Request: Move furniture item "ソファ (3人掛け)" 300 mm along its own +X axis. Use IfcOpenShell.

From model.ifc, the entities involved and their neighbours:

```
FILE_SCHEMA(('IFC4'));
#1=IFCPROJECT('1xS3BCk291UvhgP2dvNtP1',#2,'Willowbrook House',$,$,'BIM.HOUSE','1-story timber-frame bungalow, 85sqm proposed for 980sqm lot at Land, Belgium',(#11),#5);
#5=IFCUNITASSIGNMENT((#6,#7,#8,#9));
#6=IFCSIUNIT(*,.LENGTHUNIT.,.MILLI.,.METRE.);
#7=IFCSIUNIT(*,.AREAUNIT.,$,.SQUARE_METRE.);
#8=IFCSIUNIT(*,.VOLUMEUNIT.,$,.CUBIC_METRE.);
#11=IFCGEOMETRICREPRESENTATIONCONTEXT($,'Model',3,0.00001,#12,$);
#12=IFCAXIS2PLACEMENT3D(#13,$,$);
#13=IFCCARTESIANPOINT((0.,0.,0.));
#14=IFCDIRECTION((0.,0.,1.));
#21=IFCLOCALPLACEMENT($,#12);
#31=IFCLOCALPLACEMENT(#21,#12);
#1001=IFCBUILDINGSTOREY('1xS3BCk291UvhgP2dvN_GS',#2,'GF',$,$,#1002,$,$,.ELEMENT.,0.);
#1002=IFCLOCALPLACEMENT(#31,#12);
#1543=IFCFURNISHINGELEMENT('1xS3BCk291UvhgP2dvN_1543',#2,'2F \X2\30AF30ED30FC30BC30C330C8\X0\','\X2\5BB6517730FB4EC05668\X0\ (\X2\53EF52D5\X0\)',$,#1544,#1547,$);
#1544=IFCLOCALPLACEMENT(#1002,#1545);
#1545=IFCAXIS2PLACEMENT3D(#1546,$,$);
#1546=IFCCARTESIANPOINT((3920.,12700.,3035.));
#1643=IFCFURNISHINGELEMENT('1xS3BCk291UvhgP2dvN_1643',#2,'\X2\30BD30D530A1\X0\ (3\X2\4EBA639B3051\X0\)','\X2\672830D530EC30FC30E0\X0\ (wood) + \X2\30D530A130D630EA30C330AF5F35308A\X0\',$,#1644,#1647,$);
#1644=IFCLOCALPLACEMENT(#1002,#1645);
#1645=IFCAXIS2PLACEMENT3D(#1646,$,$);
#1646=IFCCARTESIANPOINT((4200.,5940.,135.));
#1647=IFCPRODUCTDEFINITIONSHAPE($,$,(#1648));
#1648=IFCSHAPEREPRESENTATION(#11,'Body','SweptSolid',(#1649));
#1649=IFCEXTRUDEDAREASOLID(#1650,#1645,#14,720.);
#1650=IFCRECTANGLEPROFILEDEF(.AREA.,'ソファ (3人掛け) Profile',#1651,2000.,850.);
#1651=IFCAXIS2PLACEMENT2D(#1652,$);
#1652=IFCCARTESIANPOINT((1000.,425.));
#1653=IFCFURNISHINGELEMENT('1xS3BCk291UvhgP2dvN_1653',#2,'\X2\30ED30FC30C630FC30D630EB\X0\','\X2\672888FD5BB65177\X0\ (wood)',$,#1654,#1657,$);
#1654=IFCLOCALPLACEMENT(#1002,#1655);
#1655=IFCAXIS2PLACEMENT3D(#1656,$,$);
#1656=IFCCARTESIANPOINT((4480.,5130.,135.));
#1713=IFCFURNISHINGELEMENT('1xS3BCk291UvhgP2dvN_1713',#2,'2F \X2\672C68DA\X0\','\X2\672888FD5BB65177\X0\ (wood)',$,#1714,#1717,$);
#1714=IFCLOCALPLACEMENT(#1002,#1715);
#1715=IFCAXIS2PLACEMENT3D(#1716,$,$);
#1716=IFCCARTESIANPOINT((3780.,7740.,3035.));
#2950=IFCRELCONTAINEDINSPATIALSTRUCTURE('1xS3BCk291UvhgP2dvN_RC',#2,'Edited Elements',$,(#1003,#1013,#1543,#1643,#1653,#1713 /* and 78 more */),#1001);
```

```python
import ifcopenshell
import ifcopenshell.api.geometry
import ifcopenshell.util.placement
import ifcopenshell.util.unit

model = ifcopenshell.open("model.ifc")
unit_scale = ifcopenshell.util.unit.calculate_unit_scale(model)

item = model.by_guid("1xS3BCk291UvhgP2dvN_1643")
matrix = ifcopenshell.util.placement.get_local_placement(item.ObjectPlacement)
matrix[:3, 3] += matrix[:3, 0] * 0.3 / unit_scale
ifcopenshell.api.geometry.edit_object_placement(model, product=item, matrix=matrix, is_si=False)

print(ifcopenshell.util.placement.get_local_placement(item.ObjectPlacement).round(3) + 0.0)

model.write("model_rev.ifc")
```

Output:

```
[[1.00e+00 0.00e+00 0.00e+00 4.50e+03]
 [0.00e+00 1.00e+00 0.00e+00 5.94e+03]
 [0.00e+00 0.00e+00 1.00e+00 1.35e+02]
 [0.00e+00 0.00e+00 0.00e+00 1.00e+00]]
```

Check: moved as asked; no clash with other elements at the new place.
